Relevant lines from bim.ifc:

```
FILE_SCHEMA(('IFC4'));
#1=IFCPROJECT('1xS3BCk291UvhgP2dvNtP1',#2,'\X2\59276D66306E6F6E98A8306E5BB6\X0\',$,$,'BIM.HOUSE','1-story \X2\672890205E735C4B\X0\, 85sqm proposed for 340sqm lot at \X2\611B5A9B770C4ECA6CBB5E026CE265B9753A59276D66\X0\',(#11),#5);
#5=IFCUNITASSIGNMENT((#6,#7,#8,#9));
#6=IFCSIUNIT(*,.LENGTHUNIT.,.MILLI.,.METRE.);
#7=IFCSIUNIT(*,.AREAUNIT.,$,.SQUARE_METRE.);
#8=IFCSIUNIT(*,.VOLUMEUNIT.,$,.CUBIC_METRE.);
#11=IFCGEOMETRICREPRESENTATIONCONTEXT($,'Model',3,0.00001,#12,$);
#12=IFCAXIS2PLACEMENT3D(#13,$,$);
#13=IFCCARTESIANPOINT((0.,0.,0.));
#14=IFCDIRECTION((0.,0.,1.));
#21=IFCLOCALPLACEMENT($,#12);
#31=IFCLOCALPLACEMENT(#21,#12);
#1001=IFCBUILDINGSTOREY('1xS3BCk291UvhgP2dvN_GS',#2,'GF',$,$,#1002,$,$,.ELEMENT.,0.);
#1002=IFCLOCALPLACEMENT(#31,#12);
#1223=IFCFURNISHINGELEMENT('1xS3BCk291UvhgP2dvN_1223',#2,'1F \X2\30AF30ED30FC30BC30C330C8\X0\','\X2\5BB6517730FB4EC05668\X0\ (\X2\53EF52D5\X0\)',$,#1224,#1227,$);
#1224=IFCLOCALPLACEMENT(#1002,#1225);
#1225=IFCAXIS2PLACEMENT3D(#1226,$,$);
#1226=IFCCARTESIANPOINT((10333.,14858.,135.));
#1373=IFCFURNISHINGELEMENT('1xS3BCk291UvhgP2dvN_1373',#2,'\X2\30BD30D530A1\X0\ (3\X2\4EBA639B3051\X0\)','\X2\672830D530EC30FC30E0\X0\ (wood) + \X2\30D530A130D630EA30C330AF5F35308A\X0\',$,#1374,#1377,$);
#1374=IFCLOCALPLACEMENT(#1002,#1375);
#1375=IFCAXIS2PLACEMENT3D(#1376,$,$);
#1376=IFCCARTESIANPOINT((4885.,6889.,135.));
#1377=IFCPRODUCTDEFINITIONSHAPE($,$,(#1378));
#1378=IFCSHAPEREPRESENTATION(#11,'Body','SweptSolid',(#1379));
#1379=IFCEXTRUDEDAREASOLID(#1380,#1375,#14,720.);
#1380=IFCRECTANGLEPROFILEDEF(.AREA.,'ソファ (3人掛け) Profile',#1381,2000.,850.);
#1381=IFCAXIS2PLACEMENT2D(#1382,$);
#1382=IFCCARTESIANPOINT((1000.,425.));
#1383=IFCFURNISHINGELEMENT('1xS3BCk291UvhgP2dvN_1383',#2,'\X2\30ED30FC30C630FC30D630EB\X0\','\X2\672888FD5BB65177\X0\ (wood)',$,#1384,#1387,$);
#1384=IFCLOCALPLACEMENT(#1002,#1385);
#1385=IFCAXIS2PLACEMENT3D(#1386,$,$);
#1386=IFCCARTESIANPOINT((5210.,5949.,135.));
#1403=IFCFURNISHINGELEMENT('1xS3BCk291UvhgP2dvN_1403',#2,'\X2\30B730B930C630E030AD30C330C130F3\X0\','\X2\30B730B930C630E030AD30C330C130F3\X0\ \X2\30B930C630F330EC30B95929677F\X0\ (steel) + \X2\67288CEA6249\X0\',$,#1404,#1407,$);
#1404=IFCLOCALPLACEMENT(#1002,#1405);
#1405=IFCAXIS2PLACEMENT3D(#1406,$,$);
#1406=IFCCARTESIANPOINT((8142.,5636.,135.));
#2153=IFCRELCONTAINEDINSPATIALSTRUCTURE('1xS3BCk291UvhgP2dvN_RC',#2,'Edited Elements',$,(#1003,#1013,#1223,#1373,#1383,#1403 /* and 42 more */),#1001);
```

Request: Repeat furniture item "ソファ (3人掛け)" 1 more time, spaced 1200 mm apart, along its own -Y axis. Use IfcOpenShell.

```python
import ifcopenshell
import ifcopenshell.api.geometry
import ifcopenshell.api.root
import ifcopenshell.util.element
import ifcopenshell.util.placement
import ifcopenshell.util.unit

model = ifcopenshell.open("bim.ifc")
unit_scale = ifcopenshell.util.unit.calculate_unit_scale(model)


def reuse_history(source, copy):
    """copy_class also copies each property set's owner history, people and application; keep the originals."""
    for rel in copy.IsDefinedBy:
        if rel.is_a("IfcRelDefinesByProperties") and (history := rel.RelatingPropertyDefinition.OwnerHistory):
            rel.RelatingPropertyDefinition.OwnerHistory = source.OwnerHistory
            ifcopenshell.util.element.remove_deep2(model, history)


source = model.by_id(1373)
base = ifcopenshell.util.placement.get_local_placement(source.ObjectPlacement)
step = -base[:3, 1] * 1.2 / unit_scale

for i in range(1, 2):
    copy = ifcopenshell.api.root.copy_class(model, product=source)
    copy.Representation = ifcopenshell.util.element.copy_deep(
        model, source.Representation, exclude=["IfcGeometricRepresentationContext", "IfcRepresentationMap"]
    )
    reuse_history(source, copy)
    matrix = base.copy()
    matrix[:3, 3] += i * step
    print("added at", matrix[:3, 3].round(3) + 0.0)
    ifcopenshell.api.geometry.edit_object_placement(model, product=copy, matrix=matrix, is_si=False)

model.write("bim_updated.ifc")
```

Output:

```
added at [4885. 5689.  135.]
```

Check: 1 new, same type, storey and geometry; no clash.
